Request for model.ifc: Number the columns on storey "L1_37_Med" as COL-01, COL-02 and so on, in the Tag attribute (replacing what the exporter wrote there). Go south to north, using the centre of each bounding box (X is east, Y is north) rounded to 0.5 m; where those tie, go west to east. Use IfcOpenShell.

First a look at what the model holds.

```python
import ifcopenshell
import ifcopenshell.util.element
import ifcopenshell.util.placement

model = ifcopenshell.open("model.ifc")
print(model.schema)
storey = next(s for s in model.by_type("IfcBuildingStorey") if s.Name == "L1_37_Med")
columns = [e for e in ifcopenshell.util.element.get_decomposition(storey) if e.is_a("IfcColumn")]
for e in sorted(columns, key=lambda e: e.id()):
    origin = ifcopenshell.util.placement.get_local_placement(e.ObjectPlacement)[:3, 3]
    print(e.id(), e.Tag, e.Name, origin.round(2) + 0.0, sep=" | ")
```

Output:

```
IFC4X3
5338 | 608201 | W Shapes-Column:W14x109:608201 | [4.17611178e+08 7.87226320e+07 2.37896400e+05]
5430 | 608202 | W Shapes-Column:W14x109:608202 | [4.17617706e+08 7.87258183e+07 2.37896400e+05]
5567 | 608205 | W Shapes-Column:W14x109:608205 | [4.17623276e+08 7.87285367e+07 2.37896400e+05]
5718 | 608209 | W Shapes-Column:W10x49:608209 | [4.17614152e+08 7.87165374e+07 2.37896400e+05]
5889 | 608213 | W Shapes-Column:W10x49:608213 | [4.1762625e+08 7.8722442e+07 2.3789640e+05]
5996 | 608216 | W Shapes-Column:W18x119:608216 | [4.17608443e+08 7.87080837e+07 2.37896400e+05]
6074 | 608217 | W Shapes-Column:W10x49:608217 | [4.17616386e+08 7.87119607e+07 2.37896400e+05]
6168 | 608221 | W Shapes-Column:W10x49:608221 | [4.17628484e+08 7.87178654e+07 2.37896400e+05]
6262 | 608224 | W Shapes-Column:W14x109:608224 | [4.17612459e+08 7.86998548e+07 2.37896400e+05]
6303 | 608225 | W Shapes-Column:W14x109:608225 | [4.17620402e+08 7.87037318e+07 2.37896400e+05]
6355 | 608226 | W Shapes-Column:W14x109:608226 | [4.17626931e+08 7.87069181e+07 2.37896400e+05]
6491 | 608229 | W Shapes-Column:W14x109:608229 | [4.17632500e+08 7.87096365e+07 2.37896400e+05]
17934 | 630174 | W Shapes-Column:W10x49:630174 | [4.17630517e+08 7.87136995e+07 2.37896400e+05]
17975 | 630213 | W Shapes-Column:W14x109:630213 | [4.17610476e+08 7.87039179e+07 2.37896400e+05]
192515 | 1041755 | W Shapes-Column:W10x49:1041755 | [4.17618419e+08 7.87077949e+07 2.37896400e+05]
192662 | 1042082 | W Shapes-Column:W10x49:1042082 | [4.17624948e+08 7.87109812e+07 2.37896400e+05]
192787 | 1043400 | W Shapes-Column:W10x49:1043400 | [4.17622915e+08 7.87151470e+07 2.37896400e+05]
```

```python
import ifcopenshell
import ifcopenshell.geom
import ifcopenshell.util.element
import ifcopenshell.util.shape

model = ifcopenshell.open("model.ifc")
settings = ifcopenshell.geom.settings()
settings.set("use-world-coords", True)


def centre(element):
    shape = ifcopenshell.geom.create_shape(settings, element)
    return ifcopenshell.util.shape.get_bbox_centroid(shape.geometry)


storey = next(s for s in model.by_type("IfcBuildingStorey") if s.Name == "L1_37_Med")
columns = [e for e in ifcopenshell.util.element.get_decomposition(storey) if e.is_a("IfcColumn")]

# Insertion points can sit at a corner or the storey origin, so sort by the geometry (in metres).
centres = {e: centre(e) for e in columns}
columns.sort(key=lambda e: (round(centres[e][1] / 0.5), centres[e][0]))

for i, e in enumerate(columns, start=1):
    number = f"COL-{i:02d}"
    e.Tag = number
    print(e.id(), number)

model.write("model_rev.ifc")
```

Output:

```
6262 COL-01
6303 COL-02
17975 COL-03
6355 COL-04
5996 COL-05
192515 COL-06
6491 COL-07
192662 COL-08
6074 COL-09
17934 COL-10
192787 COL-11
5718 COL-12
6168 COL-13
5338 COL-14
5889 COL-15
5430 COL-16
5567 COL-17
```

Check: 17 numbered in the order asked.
